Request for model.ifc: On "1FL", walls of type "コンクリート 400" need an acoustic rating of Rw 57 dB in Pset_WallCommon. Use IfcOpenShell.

First a look at what the model holds.

```python
import ifcopenshell
import ifcopenshell.util.element

model = ifcopenshell.open("model.ifc")
print(model.schema)
storey = next(s for s in model.by_type("IfcBuildingStorey") if s.Name == "1FL")
walls = [e for e in ifcopenshell.util.element.get_decomposition(storey) if e.is_a("IfcWall")]
seen = {}
for e in walls:
    element_type = ifcopenshell.util.element.get_type(e)
    key = (element_type.Name if element_type != e and element_type else None, ifcopenshell.util.element.get_pset(e, "Pset_WallCommon", "AcousticRating"))
    seen[key] = seen.get(key, 0) + 1
for (name, value), count in sorted(seen.items(), key=str):
    print(count, "x", name, "|", value)
```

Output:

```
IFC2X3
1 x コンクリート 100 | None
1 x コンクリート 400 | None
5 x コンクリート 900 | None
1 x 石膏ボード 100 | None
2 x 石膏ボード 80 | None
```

```python
import ifcopenshell
import ifcopenshell.api.pset
import ifcopenshell.util.element

model = ifcopenshell.open("model.ifc")

storey = next(s for s in model.by_type("IfcBuildingStorey") if s.Name == "1FL")
walls = [e for e in ifcopenshell.util.element.get_decomposition(storey) if e.is_a("IfcWall")]

count = 0
for e in walls:
    element_type = ifcopenshell.util.element.get_type(e)
    if element_type in (None, e) or element_type.Name != "コンクリート 400":
        continue
    # add_pset returns the element's existing set when there is one.
    pset = ifcopenshell.api.pset.add_pset(model, product=e, name="Pset_WallCommon")
    ifcopenshell.api.pset.edit_pset(model, pset=pset, properties={"AcousticRating": "Rw 57 dB"})
    count += 1

print(count, "walls updated")

model.write("model_v2.ifc")
```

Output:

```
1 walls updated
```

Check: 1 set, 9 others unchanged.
